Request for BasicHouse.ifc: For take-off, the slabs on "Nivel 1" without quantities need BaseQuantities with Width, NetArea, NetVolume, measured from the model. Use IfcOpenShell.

First a look at what the model holds.

```python
import ifcopenshell
import ifcopenshell.util.element
import ifcopenshell.util.unit

model = ifcopenshell.open("BasicHouse.ifc")
print(model.schema)
for unit_type in ("LENGTHUNIT", "AREAUNIT", "VOLUMEUNIT"):
    print(unit_type, ifcopenshell.util.unit.calculate_unit_scale(model, unit_type))
storey = next(s for s in model.by_type("IfcBuildingStorey") if s.Name == "Nivel 1")
slabs = [e for e in ifcopenshell.util.element.get_decomposition(storey) if e.is_a("IfcSlab")]
for e in sorted(slabs, key=lambda e: e.id()):
    print(e.id(), e.is_a(), e.Name, list(ifcopenshell.util.element.get_psets(e, qtos_only=True)), sep=" | ")
```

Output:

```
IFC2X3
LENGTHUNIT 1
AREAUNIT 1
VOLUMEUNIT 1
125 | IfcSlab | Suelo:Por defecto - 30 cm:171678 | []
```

```python
import ifcopenshell
import ifcopenshell.api.pset
import ifcopenshell.geom
import ifcopenshell.util.element
import ifcopenshell.util.shape
import ifcopenshell.util.unit

model = ifcopenshell.open("BasicHouse.ifc")
unit_scale = ifcopenshell.util.unit.calculate_unit_scale(model)
area_scale = ifcopenshell.util.unit.calculate_unit_scale(model, "AREAUNIT")
volume_scale = ifcopenshell.util.unit.calculate_unit_scale(model, "VOLUMEUNIT")
settings = ifcopenshell.geom.settings()

storey = next(s for s in model.by_type("IfcBuildingStorey") if s.Name == "Nivel 1")
slabs = [e for e in ifcopenshell.util.element.get_decomposition(storey) if e.is_a("IfcSlab")]

for e in sorted(slabs, key=lambda e: e.id()):
    if ifcopenshell.util.element.get_psets(e, qtos_only=True, should_inherit=False):
        continue
    # Geometry comes back in metres, in the element's own axes.
    shape = ifcopenshell.geom.create_shape(settings, e)
    values = {
        "Width": ifcopenshell.util.shape.get_z(shape.geometry) / unit_scale,
        "NetArea": ifcopenshell.util.shape.get_footprint_area(shape.geometry) / area_scale,
        "NetVolume": ifcopenshell.util.shape.get_volume(shape.geometry) / volume_scale,
    }
    qto = ifcopenshell.api.pset.add_qto(model, product=e, name="BaseQuantities")
    ifcopenshell.api.pset.edit_qto(model, qto=qto, properties=values)
    print(e.id(), {k: round(v, 3) for k, v in values.items()})

model.write("BasicHouse_v2.ifc")
```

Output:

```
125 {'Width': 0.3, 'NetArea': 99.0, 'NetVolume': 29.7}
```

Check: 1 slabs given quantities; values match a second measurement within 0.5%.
